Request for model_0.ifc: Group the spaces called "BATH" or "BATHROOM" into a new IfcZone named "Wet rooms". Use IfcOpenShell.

First a look at what the model holds.

```python
import ifcopenshell

model = ifcopenshell.open("model_0.ifc")
print(model.schema)
seen = {}
for space in model.by_type("IfcSpace"):
    seen[space.LongName] = seen.get(space.LongName, 0) + 1
for name, count in sorted(seen.items(), key=str):
    print(count, "x", name)
print("zones:", [z.Name for z in model.by_type("IfcZone")][:20])
```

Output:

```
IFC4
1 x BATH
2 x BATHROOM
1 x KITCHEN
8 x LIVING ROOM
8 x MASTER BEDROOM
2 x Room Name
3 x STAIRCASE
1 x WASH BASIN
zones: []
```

```python
import ifcopenshell
import ifcopenshell.api.group
import ifcopenshell.api.root

model = ifcopenshell.open("model_0.ifc")

names = {"BATH", "BATHROOM"}
spaces = [s for s in model.by_type("IfcSpace") if s.LongName in names]

zone = ifcopenshell.api.root.create_entity(model, ifc_class="IfcZone", name="Wet rooms")
ifcopenshell.api.group.assign_group(model, products=spaces, group=zone)
print(len(spaces), "spaces in", zone.Name)

model.write("model_0_v2.ifc")
```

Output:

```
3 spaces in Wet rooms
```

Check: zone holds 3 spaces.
